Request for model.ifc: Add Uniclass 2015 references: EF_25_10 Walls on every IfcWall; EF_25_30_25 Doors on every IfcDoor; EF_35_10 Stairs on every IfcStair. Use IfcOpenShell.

First a look at what the model holds.

```python
import ifcopenshell

model = ifcopenshell.open("model.ifc")
print(model.schema)
print("classifications:", [c.Name for c in model.by_type("IfcClassification")])
for ifc_class in ("IfcDoor", "IfcRoof", "IfcStair", "IfcWall", "IfcWindow"):
    print(ifc_class, len(model.by_type(ifc_class)))
```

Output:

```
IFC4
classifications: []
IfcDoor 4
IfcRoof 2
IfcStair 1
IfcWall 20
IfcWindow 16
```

```python
import ifcopenshell
import ifcopenshell.api.classification

model = ifcopenshell.open("model.ifc")

system = ifcopenshell.api.classification.add_classification(model, classification="Uniclass 2015")

codes = {
    "IfcWall": ("EF_25_10", "Walls"),
    "IfcDoor": ("EF_25_30_25", "Doors"),
    "IfcStair": ("EF_35_10", "Stairs"),
}
for ifc_class, (code, name) in codes.items():
    products = model.by_type(ifc_class)
    ifcopenshell.api.classification.add_reference(
        model, products=products, classification=system, identification=code, name=name
    )
    print(code, len(products))

model.write("model_rev.ifc")
```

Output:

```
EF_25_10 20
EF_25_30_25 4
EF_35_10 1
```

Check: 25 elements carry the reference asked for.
